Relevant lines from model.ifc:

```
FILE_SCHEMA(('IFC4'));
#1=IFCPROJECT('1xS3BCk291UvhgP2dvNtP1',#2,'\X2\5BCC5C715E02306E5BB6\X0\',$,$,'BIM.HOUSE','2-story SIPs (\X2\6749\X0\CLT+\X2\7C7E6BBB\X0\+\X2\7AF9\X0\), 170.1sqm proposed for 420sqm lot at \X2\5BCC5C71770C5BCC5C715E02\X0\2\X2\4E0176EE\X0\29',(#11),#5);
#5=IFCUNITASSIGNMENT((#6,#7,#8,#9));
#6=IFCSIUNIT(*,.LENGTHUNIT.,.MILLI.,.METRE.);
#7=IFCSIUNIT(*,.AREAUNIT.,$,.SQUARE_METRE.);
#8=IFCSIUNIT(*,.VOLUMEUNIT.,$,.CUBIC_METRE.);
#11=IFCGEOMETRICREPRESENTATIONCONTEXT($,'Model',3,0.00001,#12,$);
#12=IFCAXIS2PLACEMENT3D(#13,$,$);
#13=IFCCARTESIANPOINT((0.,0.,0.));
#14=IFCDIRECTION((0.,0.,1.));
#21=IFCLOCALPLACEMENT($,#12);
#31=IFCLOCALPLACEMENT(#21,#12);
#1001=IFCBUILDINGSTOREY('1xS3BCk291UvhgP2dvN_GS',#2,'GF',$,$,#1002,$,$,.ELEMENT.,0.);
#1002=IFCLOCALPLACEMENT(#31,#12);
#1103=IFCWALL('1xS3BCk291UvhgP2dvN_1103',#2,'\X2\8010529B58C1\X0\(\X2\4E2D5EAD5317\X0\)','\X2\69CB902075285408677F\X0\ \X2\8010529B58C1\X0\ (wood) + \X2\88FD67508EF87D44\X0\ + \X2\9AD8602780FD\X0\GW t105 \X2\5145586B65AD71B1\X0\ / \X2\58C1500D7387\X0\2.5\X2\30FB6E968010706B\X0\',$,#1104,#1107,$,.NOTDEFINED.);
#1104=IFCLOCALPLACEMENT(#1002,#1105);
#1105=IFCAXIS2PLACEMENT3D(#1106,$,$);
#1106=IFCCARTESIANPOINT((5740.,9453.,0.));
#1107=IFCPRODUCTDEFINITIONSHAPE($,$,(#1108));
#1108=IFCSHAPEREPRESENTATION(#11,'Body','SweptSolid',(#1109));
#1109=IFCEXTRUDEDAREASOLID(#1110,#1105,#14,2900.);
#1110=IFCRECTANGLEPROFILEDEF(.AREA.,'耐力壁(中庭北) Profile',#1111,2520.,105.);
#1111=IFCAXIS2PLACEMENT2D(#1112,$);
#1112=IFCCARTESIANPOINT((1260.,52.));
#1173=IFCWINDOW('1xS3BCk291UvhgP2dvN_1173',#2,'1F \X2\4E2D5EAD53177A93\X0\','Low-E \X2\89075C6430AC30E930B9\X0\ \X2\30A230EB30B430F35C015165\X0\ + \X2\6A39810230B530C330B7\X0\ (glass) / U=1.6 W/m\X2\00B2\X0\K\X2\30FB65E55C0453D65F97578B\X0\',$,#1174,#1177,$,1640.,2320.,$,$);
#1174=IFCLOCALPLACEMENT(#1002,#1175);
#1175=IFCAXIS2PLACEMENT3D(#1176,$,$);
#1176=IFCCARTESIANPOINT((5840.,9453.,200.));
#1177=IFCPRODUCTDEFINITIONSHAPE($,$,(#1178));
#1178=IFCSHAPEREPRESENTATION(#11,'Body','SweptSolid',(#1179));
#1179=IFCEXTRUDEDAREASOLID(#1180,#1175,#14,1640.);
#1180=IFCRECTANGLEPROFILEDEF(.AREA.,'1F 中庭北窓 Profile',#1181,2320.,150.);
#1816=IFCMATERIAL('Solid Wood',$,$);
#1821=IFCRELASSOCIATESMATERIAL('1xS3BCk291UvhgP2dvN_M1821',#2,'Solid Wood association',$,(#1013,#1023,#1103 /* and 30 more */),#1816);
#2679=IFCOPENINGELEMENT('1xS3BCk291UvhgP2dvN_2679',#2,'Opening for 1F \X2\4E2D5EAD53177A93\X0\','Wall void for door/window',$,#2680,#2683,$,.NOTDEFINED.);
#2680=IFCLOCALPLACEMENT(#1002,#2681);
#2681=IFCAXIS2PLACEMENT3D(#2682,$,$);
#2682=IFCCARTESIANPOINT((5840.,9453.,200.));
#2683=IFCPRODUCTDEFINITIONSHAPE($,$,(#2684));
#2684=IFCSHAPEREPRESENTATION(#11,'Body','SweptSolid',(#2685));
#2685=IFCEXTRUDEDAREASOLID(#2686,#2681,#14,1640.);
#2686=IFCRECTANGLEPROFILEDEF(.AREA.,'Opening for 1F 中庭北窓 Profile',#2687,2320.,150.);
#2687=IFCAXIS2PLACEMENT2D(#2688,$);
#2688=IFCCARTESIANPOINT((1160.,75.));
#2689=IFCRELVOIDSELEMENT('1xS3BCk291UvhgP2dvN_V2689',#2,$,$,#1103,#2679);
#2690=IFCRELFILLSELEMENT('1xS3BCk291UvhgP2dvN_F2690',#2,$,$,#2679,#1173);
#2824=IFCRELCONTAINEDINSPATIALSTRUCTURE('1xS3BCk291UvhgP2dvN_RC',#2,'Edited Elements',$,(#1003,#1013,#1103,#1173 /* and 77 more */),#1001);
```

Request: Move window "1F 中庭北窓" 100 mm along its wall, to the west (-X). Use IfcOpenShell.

```python
import ifcopenshell
import ifcopenshell.api.geometry
import ifcopenshell.util.placement

model = ifcopenshell.open("model.ifc")

window = model.by_id(1173)
opening = window.FillsVoids[0].RelatingOpeningElement
wall = opening.VoidsElements[0].RelatingBuildingElement

wall_matrix = ifcopenshell.util.placement.get_local_placement(wall.ObjectPlacement)
shift = wall_matrix[:3, 0] * -100.0
before = ifcopenshell.util.placement.get_local_placement(window.ObjectPlacement)[:3, 3].copy()

# The window is not placed relative to its opening, so move both.
for product in (opening, window):
    matrix = ifcopenshell.util.placement.get_local_placement(product.ObjectPlacement)
    matrix[:3, 3] += shift
    ifcopenshell.api.geometry.edit_object_placement(model, product=product, matrix=matrix, is_si=False)

after = ifcopenshell.util.placement.get_local_placement(window.ObjectPlacement)[:3, 3]
print("window moved by", (after - before).round(3) + 0.0)

model.write("model_v2.ifc")
```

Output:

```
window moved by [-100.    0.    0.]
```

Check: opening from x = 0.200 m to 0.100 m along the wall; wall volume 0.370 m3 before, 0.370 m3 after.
